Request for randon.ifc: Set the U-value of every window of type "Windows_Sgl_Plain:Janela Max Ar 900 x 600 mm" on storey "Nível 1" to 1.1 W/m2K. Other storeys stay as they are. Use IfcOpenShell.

First a look at what the model holds.

```python
import ifcopenshell
import ifcopenshell.util.element

model = ifcopenshell.open("randon.ifc")
print(model.schema)
storey = next(s for s in model.by_type("IfcBuildingStorey") if s.Name == "Nível 1")
windows = [e for e in ifcopenshell.util.element.get_decomposition(storey) if e.is_a("IfcWindow")]
seen = {}
for e in windows:
    element_type = ifcopenshell.util.element.get_type(e)
    key = (element_type.Name if element_type != e and element_type else None, ifcopenshell.util.element.get_pset(e, "Pset_WindowCommon", "ThermalTransmittance"))
    seen[key] = seen.get(key, 0) + 1
for (name, value), count in sorted(seen.items(), key=str):
    print(count, "x", name, "|", value)
```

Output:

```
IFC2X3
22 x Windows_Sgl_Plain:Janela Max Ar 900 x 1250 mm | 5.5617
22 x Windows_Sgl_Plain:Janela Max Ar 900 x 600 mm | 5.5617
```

```python
import ifcopenshell
import ifcopenshell.api.pset
import ifcopenshell.util.element

model = ifcopenshell.open("randon.ifc")

storey = next(s for s in model.by_type("IfcBuildingStorey") if s.Name == "Nível 1")
windows = [e for e in ifcopenshell.util.element.get_decomposition(storey) if e.is_a("IfcWindow")]

count = 0
for e in windows:
    element_type = ifcopenshell.util.element.get_type(e)
    if element_type in (None, e) or element_type.Name != "Windows_Sgl_Plain:Janela Max Ar 900 x 600 mm":
        continue
    # add_pset returns the element's existing set when there is one.
    pset = ifcopenshell.api.pset.add_pset(model, product=e, name="Pset_WindowCommon")
    ifcopenshell.api.pset.edit_pset(model, pset=pset, properties={"ThermalTransmittance": 1.1})
    count += 1

print(count, "windows updated")

model.write("randon_edited.ifc")
```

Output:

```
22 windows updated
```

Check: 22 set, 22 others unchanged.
